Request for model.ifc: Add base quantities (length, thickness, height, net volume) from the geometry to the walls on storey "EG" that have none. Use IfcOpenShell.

First a look at what the model holds.

```python
import ifcopenshell
import ifcopenshell.util.element
import ifcopenshell.util.unit

model = ifcopenshell.open("model.ifc")
print(model.schema)
for unit_type in ("LENGTHUNIT", "AREAUNIT", "VOLUMEUNIT"):
    print(unit_type, ifcopenshell.util.unit.calculate_unit_scale(model, unit_type))
storey = next(s for s in model.by_type("IfcBuildingStorey") if s.Name == "EG")
walls = [e for e in ifcopenshell.util.element.get_decomposition(storey) if e.is_a("IfcWall")]
for e in sorted(walls, key=lambda e: e.id()):
    print(e.id(), e.is_a(), e.Name, list(ifcopenshell.util.element.get_psets(e, qtos_only=True)), sep=" | ")
```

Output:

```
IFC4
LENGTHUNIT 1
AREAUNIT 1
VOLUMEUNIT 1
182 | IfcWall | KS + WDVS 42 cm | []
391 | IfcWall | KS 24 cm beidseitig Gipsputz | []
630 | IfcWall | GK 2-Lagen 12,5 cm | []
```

```python
import ifcopenshell
import ifcopenshell.api.pset
import ifcopenshell.geom
import ifcopenshell.util.element
import ifcopenshell.util.shape
import ifcopenshell.util.unit

model = ifcopenshell.open("model.ifc")
unit_scale = ifcopenshell.util.unit.calculate_unit_scale(model)
volume_scale = ifcopenshell.util.unit.calculate_unit_scale(model, "VOLUMEUNIT")
settings = ifcopenshell.geom.settings()

storey = next(s for s in model.by_type("IfcBuildingStorey") if s.Name == "EG")
walls = [e for e in ifcopenshell.util.element.get_decomposition(storey) if e.is_a("IfcWall")]

for e in sorted(walls, key=lambda e: e.id()):
    if ifcopenshell.util.element.get_psets(e, qtos_only=True, should_inherit=False):
        continue
    # Geometry comes back in metres, in the element's own axes.
    shape = ifcopenshell.geom.create_shape(settings, e)
    values = {
        "Length": ifcopenshell.util.shape.get_x(shape.geometry) / unit_scale,
        "Width": ifcopenshell.util.shape.get_y(shape.geometry) / unit_scale,
        "Height": ifcopenshell.util.shape.get_z(shape.geometry) / unit_scale,
        "NetVolume": ifcopenshell.util.shape.get_volume(shape.geometry) / volume_scale,
    }
    qto = ifcopenshell.api.pset.add_qto(model, product=e, name="Qto_WallBaseQuantities")
    ifcopenshell.api.pset.edit_qto(model, qto=qto, properties=values)
    print(e.id(), {k: round(v, 3) for k, v in values.items()})

model.write("model_updated.ifc")
```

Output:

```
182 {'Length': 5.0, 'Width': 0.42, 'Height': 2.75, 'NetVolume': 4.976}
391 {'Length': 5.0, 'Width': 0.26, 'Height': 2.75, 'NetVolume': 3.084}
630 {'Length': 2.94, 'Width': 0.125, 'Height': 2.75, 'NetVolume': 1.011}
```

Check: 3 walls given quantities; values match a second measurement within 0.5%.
